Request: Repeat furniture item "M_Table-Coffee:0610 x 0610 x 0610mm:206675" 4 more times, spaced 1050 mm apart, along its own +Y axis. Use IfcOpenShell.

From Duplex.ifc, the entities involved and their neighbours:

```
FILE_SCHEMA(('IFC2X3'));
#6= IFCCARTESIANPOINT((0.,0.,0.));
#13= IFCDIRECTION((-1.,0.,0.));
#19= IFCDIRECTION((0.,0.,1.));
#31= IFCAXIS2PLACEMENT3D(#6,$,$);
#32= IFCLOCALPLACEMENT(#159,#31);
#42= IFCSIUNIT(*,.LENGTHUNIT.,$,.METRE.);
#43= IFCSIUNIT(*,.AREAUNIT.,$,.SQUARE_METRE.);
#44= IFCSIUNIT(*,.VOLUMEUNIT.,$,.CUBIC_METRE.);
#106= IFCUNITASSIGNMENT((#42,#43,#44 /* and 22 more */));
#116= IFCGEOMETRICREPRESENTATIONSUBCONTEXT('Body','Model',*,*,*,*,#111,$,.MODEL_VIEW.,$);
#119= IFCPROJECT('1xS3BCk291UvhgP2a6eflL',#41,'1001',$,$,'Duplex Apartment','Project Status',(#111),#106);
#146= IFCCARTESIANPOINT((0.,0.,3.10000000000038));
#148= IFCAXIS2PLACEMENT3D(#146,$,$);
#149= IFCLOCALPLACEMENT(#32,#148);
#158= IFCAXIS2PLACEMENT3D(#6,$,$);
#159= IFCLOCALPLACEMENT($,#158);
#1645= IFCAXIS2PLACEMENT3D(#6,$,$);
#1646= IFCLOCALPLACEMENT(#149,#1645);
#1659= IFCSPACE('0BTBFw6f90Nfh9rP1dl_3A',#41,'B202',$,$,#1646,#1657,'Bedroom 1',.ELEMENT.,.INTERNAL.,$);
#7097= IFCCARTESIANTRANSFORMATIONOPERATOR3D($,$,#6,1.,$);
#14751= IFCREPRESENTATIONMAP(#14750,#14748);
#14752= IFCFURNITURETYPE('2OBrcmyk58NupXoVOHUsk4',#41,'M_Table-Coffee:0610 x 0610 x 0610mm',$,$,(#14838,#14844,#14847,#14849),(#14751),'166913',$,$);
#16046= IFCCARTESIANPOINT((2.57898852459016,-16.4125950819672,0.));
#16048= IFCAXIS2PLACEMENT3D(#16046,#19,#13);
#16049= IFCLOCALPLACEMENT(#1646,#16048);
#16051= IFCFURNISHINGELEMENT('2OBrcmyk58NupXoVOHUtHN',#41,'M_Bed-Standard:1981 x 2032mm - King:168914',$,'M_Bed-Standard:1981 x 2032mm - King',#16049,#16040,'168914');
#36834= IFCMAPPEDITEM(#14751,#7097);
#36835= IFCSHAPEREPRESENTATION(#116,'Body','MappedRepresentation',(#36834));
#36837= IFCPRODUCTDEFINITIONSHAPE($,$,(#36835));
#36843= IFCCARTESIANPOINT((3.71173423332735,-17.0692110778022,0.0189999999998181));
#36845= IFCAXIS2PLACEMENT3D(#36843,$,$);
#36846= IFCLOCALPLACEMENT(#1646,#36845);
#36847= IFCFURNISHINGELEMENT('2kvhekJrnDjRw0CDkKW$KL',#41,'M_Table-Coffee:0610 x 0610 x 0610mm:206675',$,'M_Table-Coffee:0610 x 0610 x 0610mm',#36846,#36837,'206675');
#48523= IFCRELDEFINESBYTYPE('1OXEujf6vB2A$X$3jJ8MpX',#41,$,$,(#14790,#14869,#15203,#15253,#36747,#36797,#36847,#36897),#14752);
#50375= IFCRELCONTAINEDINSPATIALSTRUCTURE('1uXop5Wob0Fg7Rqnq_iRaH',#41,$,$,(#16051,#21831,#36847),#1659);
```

```python
import ifcopenshell
import ifcopenshell.api.geometry
import ifcopenshell.api.root
import ifcopenshell.util.element
import ifcopenshell.util.placement
import ifcopenshell.util.unit

model = ifcopenshell.open("Duplex.ifc")
unit_scale = ifcopenshell.util.unit.calculate_unit_scale(model)


def reuse_history(source, copy):
    """copy_class also copies each property set's owner history, people and application; keep the originals."""
    for rel in copy.IsDefinedBy:
        if rel.is_a("IfcRelDefinesByProperties") and (history := rel.RelatingPropertyDefinition.OwnerHistory):
            rel.RelatingPropertyDefinition.OwnerHistory = source.OwnerHistory
            ifcopenshell.util.element.remove_deep2(model, history)


source = model.by_guid("2kvhekJrnDjRw0CDkKW$KL")
base = ifcopenshell.util.placement.get_local_placement(source.ObjectPlacement)
step = base[:3, 1] * 1.05 / unit_scale

for i in range(1, 5):
    copy = ifcopenshell.api.root.copy_class(model, product=source)
    copy.Representation = ifcopenshell.util.element.copy_deep(
        model, source.Representation, exclude=["IfcGeometricRepresentationContext", "IfcRepresentationMap"]
    )
    copy.Name = "M_Table-Coffee:0610 x 0610 x 0610mm"
    copy.Tag = None
    reuse_history(source, copy)
    matrix = base.copy()
    matrix[:3, 3] += i * step
    print("added at", matrix[:3, 3].round(3) + 0.0)
    ifcopenshell.api.geometry.edit_object_placement(model, product=copy, matrix=matrix, is_si=False)

model.write("Duplex-out.ifc")
```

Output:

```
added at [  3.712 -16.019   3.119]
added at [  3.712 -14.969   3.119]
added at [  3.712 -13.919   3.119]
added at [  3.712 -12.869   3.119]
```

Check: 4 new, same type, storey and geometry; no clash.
